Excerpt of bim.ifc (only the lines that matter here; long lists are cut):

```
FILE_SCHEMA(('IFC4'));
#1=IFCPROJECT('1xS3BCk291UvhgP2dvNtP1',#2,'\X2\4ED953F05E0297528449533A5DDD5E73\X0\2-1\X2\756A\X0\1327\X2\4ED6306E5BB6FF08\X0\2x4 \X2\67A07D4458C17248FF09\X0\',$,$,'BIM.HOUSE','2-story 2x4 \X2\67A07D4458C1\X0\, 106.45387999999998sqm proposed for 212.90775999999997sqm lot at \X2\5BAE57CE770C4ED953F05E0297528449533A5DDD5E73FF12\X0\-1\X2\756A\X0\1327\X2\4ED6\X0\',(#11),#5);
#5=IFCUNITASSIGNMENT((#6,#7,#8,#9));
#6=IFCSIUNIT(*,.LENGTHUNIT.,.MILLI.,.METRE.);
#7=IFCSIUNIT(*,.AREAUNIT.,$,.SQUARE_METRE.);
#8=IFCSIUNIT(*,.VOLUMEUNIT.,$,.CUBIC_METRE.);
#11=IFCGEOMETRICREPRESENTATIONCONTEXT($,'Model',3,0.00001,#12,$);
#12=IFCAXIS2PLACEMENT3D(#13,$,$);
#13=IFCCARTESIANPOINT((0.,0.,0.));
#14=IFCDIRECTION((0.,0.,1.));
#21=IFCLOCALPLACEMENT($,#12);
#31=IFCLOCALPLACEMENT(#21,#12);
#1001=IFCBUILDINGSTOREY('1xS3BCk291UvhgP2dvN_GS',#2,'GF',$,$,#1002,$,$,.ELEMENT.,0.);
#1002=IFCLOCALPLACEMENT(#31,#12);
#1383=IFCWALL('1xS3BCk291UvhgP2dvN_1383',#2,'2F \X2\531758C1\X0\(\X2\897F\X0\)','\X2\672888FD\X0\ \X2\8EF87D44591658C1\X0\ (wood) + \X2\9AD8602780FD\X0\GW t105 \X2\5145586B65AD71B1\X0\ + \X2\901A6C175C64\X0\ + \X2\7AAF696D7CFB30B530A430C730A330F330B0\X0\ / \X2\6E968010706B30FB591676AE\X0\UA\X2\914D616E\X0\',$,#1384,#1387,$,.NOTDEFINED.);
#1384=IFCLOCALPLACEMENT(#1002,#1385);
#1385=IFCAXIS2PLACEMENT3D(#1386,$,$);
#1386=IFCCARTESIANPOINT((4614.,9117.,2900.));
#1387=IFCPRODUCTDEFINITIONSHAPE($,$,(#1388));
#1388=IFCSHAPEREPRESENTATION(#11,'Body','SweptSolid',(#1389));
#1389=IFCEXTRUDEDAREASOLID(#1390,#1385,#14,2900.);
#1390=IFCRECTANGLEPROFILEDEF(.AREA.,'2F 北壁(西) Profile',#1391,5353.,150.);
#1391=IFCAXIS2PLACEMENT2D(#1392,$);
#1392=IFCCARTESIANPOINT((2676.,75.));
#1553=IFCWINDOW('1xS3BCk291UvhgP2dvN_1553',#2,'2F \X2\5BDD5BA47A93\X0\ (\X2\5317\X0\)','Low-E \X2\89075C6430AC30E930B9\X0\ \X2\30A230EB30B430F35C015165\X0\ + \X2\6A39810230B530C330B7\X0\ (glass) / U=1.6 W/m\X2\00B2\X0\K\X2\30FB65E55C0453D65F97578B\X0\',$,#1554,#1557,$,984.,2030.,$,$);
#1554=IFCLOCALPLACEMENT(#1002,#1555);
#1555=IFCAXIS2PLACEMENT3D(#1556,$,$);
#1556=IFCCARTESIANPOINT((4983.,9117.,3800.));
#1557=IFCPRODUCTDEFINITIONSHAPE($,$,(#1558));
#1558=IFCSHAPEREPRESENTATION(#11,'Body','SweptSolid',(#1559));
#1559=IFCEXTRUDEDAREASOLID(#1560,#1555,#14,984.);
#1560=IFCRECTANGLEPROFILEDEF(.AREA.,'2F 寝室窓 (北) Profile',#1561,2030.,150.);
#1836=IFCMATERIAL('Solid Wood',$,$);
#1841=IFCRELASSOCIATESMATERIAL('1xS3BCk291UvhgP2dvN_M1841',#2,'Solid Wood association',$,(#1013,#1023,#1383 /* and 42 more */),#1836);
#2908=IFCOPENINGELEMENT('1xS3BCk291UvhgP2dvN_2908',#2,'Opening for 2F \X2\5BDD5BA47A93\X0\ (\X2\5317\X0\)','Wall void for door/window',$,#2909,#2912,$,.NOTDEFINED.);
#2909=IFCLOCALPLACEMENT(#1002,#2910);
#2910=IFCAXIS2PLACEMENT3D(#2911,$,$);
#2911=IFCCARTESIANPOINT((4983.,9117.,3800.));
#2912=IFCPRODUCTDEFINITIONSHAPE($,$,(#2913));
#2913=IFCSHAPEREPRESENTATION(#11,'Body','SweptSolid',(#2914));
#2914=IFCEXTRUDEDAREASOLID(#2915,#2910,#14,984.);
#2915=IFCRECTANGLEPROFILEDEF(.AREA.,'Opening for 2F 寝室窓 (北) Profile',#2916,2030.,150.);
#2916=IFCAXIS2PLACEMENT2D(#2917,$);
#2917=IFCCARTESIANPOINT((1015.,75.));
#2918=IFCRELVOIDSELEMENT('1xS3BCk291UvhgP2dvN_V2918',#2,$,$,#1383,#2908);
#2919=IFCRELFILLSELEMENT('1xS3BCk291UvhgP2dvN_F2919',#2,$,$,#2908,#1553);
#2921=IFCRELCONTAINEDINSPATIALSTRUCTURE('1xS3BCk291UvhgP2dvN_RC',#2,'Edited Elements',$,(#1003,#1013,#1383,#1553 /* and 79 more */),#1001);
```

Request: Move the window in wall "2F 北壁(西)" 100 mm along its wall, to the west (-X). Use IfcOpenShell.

```python
import ifcopenshell
import ifcopenshell.api.geometry
import ifcopenshell.util.placement
import ifcopenshell.util.unit

model = ifcopenshell.open("bim.ifc")
unit_scale = ifcopenshell.util.unit.calculate_unit_scale(model)

window = model.by_id(1553)
opening = window.FillsVoids[0].RelatingOpeningElement
wall = opening.VoidsElements[0].RelatingBuildingElement

wall_matrix = ifcopenshell.util.placement.get_local_placement(wall.ObjectPlacement)
shift = wall_matrix[:3, 0] * -0.1 / unit_scale
before = ifcopenshell.util.placement.get_local_placement(window.ObjectPlacement)[:3, 3].copy()

# The window is not placed relative to its opening, so move both.
for product in (opening, window):
    matrix = ifcopenshell.util.placement.get_local_placement(product.ObjectPlacement)
    matrix[:3, 3] += shift
    ifcopenshell.api.geometry.edit_object_placement(model, product=product, matrix=matrix, is_si=False)

after = ifcopenshell.util.placement.get_local_placement(window.ObjectPlacement)[:3, 3]
print("window moved by", (after - before).round(3) + 0.0)

model.write("bim_rev.ifc")
```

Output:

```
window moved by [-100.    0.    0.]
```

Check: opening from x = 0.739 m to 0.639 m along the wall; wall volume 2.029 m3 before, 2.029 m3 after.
